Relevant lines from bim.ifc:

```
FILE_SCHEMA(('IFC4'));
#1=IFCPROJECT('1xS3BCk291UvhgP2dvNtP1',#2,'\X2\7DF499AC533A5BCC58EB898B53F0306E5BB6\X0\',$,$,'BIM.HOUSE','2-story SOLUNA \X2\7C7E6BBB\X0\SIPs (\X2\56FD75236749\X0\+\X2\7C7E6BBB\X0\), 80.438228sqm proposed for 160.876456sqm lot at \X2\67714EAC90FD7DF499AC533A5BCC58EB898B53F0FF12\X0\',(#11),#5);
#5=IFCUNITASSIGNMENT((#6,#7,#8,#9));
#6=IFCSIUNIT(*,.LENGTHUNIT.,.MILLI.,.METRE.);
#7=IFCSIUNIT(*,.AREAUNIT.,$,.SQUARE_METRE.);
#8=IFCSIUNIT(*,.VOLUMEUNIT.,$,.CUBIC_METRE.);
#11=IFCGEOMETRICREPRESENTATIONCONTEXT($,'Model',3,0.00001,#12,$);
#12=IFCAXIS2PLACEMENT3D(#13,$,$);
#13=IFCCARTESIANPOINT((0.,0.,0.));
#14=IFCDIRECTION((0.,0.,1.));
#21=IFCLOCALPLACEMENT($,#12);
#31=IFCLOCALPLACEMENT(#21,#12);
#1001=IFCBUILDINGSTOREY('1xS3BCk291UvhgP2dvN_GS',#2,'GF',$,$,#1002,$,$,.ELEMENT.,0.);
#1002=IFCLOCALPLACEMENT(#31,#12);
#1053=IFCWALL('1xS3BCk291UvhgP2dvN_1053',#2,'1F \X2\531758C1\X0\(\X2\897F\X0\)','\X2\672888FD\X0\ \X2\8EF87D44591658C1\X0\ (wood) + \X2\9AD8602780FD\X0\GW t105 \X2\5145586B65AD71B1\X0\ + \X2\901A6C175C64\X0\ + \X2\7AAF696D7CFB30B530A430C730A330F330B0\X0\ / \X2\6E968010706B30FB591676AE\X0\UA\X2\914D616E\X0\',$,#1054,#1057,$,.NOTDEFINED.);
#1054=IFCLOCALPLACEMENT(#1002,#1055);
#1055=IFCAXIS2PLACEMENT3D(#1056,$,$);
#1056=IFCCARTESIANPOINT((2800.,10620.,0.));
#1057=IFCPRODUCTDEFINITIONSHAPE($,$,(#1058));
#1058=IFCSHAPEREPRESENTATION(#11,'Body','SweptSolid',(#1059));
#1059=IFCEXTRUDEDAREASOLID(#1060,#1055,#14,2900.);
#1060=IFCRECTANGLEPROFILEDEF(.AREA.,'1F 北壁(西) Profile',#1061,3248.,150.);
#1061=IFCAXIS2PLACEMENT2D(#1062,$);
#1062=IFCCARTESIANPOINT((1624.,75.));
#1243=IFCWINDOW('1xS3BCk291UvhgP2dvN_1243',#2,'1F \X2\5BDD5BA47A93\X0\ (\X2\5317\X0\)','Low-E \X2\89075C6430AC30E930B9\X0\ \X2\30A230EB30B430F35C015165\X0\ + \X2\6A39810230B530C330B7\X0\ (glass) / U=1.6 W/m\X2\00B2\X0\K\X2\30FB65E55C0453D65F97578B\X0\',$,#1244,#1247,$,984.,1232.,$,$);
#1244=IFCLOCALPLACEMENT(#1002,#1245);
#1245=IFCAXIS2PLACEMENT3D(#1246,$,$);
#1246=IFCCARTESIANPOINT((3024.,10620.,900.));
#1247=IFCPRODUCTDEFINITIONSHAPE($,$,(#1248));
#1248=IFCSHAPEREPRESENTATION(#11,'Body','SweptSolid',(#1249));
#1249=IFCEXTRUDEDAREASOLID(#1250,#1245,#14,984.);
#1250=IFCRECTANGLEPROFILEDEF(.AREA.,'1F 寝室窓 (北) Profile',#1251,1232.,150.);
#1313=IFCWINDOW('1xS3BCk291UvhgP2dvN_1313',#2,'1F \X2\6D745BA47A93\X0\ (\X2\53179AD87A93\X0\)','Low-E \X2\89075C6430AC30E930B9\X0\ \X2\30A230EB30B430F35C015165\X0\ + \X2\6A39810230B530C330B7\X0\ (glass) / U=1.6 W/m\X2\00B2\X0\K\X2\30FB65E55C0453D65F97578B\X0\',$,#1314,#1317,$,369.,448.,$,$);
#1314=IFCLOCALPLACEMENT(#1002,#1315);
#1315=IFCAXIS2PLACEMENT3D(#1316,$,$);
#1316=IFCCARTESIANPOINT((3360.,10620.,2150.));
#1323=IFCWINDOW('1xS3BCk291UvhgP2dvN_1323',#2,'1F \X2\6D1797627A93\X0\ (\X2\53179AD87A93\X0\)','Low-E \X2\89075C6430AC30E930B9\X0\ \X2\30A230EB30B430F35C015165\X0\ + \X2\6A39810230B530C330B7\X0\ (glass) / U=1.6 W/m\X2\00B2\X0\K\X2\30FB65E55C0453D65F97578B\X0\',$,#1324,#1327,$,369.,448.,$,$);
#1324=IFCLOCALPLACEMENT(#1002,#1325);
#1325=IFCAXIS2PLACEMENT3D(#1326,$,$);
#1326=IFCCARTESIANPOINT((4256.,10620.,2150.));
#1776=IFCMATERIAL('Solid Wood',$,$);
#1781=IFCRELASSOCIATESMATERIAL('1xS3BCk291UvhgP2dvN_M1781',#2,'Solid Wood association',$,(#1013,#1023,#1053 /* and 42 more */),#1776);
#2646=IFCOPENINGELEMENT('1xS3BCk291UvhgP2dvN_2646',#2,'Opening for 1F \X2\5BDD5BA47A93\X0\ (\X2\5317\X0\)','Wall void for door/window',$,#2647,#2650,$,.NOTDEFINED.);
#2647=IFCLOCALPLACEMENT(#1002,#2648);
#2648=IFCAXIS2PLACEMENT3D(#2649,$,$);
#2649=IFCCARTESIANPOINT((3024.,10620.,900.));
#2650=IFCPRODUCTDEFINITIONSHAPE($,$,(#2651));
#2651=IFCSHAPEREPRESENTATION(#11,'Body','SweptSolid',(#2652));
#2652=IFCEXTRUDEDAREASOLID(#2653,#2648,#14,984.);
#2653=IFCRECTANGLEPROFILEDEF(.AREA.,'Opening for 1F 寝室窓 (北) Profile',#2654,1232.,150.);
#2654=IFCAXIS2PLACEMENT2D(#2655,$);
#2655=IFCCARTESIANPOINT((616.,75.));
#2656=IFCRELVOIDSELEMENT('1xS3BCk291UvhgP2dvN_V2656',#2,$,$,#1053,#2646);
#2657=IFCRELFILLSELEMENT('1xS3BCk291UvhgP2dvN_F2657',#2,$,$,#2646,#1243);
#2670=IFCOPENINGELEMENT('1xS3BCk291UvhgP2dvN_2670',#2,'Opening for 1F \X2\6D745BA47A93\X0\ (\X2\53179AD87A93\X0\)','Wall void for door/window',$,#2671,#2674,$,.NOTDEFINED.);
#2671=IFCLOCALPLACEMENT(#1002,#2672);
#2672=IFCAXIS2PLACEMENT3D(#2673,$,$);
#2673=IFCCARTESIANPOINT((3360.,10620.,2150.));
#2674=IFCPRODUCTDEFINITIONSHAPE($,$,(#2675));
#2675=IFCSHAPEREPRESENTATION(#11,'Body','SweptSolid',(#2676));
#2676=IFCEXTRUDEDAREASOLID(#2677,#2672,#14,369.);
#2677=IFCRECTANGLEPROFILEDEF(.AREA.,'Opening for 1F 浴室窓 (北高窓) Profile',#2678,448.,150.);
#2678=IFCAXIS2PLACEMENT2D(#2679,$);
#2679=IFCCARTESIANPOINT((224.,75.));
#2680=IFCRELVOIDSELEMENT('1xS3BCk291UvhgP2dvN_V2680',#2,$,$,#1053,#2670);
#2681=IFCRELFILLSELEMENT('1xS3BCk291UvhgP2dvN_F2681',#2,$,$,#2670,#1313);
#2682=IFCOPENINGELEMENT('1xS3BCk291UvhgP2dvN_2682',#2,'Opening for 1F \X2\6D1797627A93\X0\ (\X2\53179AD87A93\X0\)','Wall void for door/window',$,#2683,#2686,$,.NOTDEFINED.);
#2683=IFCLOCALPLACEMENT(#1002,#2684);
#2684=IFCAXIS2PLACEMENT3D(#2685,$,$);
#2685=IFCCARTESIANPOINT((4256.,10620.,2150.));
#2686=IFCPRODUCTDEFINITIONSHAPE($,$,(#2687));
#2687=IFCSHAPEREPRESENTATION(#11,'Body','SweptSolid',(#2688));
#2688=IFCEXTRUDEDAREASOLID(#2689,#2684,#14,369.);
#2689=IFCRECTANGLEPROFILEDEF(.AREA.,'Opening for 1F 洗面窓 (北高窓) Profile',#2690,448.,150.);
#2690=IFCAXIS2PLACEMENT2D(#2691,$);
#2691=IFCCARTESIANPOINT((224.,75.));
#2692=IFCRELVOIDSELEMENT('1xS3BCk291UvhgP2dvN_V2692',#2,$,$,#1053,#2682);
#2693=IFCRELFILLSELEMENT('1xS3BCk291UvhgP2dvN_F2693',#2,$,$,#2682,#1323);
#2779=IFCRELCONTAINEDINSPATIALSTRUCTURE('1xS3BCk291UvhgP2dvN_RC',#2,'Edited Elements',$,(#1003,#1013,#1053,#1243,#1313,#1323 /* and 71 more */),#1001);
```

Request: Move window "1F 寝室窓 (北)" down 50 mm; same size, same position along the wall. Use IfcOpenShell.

```python
import numpy as np
import ifcopenshell
import ifcopenshell.api.geometry
import ifcopenshell.util.placement
import ifcopenshell.util.unit

model = ifcopenshell.open("bim.ifc")
unit_scale = ifcopenshell.util.unit.calculate_unit_scale(model)

window = model.by_guid("1xS3BCk291UvhgP2dvN_1243")
opening = window.FillsVoids[0].RelatingOpeningElement
dz = -50.0

shift = np.array([0.0, 0.0, dz])
# The window is not placed relative to its opening, so move both.
for product in (opening, window):
    matrix = ifcopenshell.util.placement.get_local_placement(product.ObjectPlacement)
    matrix[:3, 3] += shift
    ifcopenshell.api.geometry.edit_object_placement(model, product=product, matrix=matrix, is_si=False)

print(f"moved by {dz * unit_scale:+.3f} m")

model.write("bim_updated.ifc")
```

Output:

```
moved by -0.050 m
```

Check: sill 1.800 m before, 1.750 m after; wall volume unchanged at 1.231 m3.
